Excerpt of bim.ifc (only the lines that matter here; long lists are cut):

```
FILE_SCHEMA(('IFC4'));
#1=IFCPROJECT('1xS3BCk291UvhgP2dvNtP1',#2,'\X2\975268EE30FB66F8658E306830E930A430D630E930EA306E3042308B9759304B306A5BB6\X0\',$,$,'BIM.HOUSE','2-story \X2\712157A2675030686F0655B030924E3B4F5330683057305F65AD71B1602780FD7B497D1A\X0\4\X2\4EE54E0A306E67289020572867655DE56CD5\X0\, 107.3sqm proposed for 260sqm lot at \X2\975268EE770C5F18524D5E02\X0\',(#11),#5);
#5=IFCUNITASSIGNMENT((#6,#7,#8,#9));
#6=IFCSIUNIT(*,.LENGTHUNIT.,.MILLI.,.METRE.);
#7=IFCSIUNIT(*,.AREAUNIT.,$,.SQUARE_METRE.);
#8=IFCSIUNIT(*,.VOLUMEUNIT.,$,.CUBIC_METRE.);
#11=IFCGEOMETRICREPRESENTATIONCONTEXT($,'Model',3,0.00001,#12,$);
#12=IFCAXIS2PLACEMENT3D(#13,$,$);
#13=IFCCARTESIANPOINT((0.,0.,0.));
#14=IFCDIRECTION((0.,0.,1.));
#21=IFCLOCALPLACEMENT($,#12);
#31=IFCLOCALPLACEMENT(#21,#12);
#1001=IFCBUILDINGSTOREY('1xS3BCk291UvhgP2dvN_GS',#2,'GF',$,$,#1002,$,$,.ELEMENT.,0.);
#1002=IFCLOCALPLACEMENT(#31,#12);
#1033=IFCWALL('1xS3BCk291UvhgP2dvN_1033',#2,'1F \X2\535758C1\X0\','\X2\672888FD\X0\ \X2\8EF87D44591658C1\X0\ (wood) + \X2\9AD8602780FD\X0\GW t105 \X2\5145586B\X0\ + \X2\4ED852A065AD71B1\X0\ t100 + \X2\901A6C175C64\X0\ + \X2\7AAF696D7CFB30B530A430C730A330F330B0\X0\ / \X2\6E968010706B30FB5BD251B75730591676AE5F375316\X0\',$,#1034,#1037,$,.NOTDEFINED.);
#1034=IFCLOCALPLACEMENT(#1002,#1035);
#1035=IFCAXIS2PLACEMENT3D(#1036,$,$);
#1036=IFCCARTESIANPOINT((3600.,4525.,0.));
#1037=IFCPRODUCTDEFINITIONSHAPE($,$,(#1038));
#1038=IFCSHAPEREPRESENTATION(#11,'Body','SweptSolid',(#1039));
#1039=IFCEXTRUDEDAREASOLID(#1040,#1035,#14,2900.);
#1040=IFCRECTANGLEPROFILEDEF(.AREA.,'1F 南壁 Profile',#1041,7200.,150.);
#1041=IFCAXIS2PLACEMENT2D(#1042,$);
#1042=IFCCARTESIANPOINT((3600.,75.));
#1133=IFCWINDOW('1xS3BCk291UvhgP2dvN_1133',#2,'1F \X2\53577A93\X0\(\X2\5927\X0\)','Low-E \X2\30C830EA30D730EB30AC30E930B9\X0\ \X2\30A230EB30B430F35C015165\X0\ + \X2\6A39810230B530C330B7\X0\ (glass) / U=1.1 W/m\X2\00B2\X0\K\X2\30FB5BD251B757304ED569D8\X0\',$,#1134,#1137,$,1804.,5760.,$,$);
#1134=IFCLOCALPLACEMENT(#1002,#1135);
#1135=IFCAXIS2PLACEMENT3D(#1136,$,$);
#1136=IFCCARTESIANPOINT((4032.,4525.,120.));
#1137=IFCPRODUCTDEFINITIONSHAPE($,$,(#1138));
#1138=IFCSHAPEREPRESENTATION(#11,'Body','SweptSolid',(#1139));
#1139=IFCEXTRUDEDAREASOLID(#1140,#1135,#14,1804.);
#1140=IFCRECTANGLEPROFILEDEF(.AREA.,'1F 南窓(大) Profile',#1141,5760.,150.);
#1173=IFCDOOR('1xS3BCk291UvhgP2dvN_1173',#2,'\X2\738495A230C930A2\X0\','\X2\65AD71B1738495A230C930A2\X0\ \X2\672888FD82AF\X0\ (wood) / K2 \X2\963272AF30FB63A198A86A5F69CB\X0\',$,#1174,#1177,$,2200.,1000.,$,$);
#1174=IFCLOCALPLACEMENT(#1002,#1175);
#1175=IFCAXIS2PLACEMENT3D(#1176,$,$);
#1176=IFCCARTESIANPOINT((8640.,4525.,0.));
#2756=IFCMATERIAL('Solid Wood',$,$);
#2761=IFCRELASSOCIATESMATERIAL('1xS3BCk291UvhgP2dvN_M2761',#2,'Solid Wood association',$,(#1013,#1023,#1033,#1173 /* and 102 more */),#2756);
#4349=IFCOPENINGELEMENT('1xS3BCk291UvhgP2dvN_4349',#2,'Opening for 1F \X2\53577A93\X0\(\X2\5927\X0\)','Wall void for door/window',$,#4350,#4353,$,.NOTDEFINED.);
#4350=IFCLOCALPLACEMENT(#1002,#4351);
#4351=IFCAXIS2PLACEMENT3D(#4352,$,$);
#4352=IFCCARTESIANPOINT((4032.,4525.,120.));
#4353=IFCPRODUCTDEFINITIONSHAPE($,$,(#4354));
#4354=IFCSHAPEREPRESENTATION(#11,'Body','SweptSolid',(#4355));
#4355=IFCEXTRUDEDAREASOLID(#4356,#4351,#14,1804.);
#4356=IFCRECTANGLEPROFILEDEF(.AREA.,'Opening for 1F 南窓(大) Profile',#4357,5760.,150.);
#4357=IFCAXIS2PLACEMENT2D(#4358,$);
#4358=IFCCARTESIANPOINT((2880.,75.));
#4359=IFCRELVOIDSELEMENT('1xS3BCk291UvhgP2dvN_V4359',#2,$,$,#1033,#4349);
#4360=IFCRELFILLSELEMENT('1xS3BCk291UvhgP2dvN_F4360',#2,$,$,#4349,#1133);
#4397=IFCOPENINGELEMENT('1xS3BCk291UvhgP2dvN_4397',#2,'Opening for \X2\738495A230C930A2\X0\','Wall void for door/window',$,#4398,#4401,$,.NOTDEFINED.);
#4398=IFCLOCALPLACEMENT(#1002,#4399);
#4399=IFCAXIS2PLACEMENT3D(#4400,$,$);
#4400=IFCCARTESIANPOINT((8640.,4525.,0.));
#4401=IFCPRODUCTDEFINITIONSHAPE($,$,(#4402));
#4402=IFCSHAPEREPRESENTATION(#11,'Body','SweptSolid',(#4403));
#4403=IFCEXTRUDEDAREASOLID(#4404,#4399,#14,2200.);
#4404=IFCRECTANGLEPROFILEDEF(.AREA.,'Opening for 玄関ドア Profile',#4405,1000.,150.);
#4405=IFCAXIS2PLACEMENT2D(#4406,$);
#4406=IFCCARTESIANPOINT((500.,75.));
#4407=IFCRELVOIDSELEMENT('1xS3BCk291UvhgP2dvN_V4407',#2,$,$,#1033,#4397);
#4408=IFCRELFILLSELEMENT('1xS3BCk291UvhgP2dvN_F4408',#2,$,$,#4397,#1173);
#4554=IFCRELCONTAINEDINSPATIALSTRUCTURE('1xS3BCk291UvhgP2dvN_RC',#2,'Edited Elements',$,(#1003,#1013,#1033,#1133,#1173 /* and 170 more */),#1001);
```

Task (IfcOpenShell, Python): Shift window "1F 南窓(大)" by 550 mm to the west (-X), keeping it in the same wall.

```python
import ifcopenshell
import ifcopenshell.api.geometry
import ifcopenshell.util.placement
import ifcopenshell.util.unit

model = ifcopenshell.open("bim.ifc")
unit_scale = ifcopenshell.util.unit.calculate_unit_scale(model)

window = model.by_id(1133)
opening = window.FillsVoids[0].RelatingOpeningElement
wall = opening.VoidsElements[0].RelatingBuildingElement

wall_matrix = ifcopenshell.util.placement.get_local_placement(wall.ObjectPlacement)
shift = wall_matrix[:3, 0] * -0.55 / unit_scale
before = ifcopenshell.util.placement.get_local_placement(window.ObjectPlacement)[:3, 3].copy()

# The window is not placed relative to its opening, so move both.
for product in (opening, window):
    matrix = ifcopenshell.util.placement.get_local_placement(product.ObjectPlacement)
    matrix[:3, 3] += shift
    ifcopenshell.api.geometry.edit_object_placement(model, product=product, matrix=matrix, is_si=False)

after = ifcopenshell.util.placement.get_local_placement(window.ObjectPlacement)[:3, 3]
print("window moved by", (after - before).round(3) + 0.0)

model.write("bim_v2.ifc")
```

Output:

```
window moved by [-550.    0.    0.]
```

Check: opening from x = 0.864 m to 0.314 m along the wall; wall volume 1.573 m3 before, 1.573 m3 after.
